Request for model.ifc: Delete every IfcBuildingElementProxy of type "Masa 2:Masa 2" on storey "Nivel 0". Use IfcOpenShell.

First a look at what the model holds.

```python
import ifcopenshell
import ifcopenshell.util.element

model = ifcopenshell.open("model.ifc")
print(model.schema)
storey = next(s for s in model.by_type("IfcBuildingStorey") if s.Name == "Nivel 0")
proxies = [e for e in ifcopenshell.util.element.get_decomposition(storey) if e.is_a("IfcBuildingElementProxy")]
seen = {}
for e in proxies:
    element_type = ifcopenshell.util.element.get_type(e)
    name = element_type.Name if element_type not in (None, e) else None
    seen[name] = seen.get(name, 0) + 1
for name, count in sorted(seen.items(), key=str):
    print(count, "x", name)
```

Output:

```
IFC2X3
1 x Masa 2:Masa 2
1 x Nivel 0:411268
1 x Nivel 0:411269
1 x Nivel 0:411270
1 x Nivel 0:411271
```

```python
import ifcopenshell
import ifcopenshell.api.root
import ifcopenshell.util.element

model = ifcopenshell.open("model.ifc")

storey = next(s for s in model.by_type("IfcBuildingStorey") if s.Name == "Nivel 0")
proxies = [e for e in ifcopenshell.util.element.get_decomposition(storey) if e.is_a("IfcBuildingElementProxy")]
targets = [e for e in proxies if (t := ifcopenshell.util.element.get_type(e)) not in (None, e) and t.Name == "Masa 2:Masa 2"]

for e in targets:
    ifcopenshell.api.root.remove_product(model, product=e)
print(len(targets), "removed")

model.write("model-out.ifc")
```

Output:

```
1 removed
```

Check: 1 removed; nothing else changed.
